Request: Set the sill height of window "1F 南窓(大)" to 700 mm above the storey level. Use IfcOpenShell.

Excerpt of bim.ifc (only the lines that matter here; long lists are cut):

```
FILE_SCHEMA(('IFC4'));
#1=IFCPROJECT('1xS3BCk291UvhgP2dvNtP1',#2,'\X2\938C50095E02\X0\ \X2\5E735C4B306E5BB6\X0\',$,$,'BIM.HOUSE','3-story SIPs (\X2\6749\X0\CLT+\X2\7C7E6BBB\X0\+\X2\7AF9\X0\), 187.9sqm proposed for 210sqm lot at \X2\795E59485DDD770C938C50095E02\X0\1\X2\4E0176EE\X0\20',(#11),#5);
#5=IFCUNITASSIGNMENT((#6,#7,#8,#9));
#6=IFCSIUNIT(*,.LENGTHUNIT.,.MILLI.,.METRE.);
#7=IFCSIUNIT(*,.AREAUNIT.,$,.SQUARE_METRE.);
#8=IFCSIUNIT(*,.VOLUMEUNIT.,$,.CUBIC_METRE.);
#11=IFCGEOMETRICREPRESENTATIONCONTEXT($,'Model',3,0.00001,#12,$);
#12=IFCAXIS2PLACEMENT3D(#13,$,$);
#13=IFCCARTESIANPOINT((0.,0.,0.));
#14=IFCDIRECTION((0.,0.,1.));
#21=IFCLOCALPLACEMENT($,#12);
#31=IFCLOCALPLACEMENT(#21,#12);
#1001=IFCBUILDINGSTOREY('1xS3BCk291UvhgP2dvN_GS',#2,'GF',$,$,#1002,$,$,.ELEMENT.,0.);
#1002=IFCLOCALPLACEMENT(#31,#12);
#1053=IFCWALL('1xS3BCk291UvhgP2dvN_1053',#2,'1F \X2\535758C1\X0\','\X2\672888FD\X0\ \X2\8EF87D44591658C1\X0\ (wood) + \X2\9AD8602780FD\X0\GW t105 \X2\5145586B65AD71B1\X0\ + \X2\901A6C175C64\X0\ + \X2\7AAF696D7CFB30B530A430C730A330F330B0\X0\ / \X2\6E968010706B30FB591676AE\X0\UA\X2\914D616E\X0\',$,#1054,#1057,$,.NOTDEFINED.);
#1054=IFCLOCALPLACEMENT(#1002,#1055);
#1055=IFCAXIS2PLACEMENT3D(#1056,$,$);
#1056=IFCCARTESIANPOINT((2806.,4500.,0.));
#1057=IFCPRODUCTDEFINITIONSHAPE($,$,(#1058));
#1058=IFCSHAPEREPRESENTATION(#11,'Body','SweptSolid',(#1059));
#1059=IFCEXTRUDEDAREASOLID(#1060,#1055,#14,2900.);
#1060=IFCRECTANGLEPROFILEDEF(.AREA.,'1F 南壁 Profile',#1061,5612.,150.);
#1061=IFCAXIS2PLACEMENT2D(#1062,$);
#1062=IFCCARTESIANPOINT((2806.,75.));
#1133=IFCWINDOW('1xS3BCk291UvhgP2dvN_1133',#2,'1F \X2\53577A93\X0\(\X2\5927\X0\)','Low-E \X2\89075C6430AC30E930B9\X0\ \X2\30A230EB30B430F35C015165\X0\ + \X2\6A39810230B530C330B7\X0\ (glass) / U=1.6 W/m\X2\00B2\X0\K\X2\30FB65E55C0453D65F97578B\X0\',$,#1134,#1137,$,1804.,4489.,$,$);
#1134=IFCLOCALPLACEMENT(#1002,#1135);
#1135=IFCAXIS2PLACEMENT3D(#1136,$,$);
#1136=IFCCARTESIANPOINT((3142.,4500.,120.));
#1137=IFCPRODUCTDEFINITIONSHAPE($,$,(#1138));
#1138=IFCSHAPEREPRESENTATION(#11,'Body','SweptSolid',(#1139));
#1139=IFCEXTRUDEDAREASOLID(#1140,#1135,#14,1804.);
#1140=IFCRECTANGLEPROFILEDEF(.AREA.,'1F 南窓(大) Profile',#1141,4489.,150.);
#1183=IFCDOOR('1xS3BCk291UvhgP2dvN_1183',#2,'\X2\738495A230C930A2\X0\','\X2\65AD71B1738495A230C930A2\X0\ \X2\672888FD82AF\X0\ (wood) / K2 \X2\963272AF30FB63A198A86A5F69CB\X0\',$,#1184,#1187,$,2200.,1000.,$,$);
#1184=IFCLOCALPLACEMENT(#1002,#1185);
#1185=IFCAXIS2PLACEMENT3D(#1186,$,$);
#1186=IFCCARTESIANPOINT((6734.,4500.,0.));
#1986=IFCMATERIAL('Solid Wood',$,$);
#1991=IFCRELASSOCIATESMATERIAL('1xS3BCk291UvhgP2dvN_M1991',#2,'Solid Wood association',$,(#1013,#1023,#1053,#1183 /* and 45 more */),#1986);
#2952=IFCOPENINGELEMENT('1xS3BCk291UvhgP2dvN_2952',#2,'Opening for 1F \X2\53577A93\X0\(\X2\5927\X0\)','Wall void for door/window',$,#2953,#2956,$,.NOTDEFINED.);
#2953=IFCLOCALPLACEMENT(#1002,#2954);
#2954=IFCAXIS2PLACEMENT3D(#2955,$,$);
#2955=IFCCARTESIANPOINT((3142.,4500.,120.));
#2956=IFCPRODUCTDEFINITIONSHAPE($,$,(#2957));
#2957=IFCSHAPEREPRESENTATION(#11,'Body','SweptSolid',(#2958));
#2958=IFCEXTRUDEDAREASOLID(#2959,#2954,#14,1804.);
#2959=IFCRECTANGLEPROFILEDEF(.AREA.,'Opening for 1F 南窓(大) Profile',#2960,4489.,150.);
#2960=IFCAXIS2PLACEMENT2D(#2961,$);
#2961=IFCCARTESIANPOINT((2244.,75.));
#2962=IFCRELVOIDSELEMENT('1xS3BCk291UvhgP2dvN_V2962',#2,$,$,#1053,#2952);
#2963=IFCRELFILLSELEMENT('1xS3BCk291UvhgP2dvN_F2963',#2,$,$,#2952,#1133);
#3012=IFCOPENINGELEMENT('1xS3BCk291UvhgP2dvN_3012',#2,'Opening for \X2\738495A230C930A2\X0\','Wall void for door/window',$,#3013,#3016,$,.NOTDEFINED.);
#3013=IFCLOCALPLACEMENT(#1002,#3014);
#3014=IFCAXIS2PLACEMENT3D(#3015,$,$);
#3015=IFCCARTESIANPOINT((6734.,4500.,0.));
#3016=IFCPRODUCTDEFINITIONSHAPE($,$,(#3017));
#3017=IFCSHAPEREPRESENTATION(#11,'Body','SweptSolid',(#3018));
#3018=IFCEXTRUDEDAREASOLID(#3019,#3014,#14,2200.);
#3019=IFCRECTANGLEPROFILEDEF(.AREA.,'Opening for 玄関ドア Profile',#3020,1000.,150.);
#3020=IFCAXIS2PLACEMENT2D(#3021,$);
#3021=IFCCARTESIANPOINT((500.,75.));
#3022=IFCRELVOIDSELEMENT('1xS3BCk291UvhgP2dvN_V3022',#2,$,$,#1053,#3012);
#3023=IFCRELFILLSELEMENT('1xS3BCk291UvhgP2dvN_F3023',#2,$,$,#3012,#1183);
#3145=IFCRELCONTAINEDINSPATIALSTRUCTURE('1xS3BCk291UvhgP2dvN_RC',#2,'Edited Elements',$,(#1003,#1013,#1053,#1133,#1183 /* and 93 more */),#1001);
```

```python
import numpy as np
import ifcopenshell
import ifcopenshell.api.geometry
import ifcopenshell.geom
import ifcopenshell.util.element
import ifcopenshell.util.placement
import ifcopenshell.util.shape
import ifcopenshell.util.unit

model = ifcopenshell.open("bim.ifc")
unit_scale = ifcopenshell.util.unit.calculate_unit_scale(model)

window = model.by_guid("1xS3BCk291UvhgP2dvN_1133")
opening = window.FillsVoids[0].RelatingOpeningElement
storey = ifcopenshell.util.element.get_container(window, ifc_class="IfcBuildingStorey")
level = ifcopenshell.util.placement.get_local_placement(storey.ObjectPlacement)[2, 3]

# The opening's origin need not be at the sill, so measure its lowest point.
shape = ifcopenshell.geom.create_shape(ifcopenshell.geom.settings(), opening)
bottom = ifcopenshell.util.shape.get_shape_bottom_elevation(shape, shape.geometry) / unit_scale
dz = level + 700.0 - bottom

shift = np.array([0.0, 0.0, dz])
# The window is not placed relative to its opening, so move both.
for product in (opening, window):
    matrix = ifcopenshell.util.placement.get_local_placement(product.ObjectPlacement)
    matrix[:3, 3] += shift
    ifcopenshell.api.geometry.edit_object_placement(model, product=product, matrix=matrix, is_si=False)

print(f"moved by {dz * unit_scale:+.3f} m")

model.write("bim-out.ifc")
```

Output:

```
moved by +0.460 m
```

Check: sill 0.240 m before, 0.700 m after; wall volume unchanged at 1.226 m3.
